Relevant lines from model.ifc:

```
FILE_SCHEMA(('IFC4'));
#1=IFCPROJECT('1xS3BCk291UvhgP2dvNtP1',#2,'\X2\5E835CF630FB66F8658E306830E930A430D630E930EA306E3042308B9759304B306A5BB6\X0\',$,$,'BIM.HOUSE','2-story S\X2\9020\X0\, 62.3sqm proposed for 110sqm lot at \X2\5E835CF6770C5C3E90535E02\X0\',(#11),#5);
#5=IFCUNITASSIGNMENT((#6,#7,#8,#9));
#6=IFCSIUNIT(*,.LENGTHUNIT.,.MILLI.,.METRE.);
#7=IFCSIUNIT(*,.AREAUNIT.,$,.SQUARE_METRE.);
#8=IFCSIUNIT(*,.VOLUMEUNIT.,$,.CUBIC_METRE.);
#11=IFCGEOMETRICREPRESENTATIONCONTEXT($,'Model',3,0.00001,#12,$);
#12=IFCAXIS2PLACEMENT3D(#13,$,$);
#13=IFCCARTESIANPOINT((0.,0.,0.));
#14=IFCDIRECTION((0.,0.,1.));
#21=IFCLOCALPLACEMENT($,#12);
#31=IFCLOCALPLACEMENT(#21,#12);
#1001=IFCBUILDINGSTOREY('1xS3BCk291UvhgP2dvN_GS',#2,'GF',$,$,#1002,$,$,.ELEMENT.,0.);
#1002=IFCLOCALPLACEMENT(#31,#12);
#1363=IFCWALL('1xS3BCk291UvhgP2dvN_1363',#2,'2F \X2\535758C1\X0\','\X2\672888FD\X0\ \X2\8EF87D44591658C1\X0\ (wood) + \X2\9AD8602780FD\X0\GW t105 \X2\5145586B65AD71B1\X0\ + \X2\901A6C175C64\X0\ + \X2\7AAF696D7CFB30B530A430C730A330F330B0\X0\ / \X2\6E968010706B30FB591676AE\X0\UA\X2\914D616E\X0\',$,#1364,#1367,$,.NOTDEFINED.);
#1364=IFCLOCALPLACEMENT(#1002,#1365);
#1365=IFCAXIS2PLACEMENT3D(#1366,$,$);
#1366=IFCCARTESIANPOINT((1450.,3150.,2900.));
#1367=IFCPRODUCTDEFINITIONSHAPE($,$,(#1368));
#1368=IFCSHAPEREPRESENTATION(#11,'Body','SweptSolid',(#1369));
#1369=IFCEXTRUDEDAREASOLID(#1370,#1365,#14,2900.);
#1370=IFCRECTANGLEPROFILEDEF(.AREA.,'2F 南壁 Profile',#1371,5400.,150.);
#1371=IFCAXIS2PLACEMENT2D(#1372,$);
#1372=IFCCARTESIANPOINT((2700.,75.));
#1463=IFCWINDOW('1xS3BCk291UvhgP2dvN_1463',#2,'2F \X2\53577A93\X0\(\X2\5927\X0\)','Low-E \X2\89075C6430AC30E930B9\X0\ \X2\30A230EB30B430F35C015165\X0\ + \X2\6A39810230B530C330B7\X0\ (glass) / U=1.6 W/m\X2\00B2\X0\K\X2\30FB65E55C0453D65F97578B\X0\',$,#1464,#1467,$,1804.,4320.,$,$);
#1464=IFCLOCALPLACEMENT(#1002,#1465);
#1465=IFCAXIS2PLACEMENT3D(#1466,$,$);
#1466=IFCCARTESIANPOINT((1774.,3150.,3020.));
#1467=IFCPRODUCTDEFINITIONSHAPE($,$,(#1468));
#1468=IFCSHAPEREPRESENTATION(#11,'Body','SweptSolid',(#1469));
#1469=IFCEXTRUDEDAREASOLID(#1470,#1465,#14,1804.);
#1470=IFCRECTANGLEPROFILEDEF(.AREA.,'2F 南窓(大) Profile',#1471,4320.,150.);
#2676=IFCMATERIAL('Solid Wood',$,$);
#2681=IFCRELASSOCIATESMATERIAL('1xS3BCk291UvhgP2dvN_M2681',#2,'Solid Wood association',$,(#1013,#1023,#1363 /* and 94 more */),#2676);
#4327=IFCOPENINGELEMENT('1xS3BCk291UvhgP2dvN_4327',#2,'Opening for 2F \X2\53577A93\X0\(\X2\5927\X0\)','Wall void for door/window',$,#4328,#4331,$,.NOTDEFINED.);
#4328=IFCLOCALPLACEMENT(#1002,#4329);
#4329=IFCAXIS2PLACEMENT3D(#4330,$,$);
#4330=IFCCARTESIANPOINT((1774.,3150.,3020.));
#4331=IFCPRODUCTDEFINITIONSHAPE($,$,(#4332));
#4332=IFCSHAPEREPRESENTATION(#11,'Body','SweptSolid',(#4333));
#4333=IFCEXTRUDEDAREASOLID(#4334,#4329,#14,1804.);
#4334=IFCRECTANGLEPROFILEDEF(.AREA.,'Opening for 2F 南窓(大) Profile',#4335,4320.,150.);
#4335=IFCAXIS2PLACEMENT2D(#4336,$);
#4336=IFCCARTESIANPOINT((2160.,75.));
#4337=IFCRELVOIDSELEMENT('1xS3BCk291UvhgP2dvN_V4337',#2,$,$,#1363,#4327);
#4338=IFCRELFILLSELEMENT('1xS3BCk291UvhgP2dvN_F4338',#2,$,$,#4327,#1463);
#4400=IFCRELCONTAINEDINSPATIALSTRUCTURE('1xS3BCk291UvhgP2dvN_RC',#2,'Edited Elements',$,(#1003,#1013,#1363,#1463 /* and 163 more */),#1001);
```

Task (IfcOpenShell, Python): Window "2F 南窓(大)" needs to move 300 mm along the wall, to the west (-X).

```python
import ifcopenshell
import ifcopenshell.api.geometry
import ifcopenshell.util.placement
import ifcopenshell.util.unit

model = ifcopenshell.open("model.ifc")
unit_scale = ifcopenshell.util.unit.calculate_unit_scale(model)

window = model.by_guid("1xS3BCk291UvhgP2dvN_1463")
opening = window.FillsVoids[0].RelatingOpeningElement
wall = opening.VoidsElements[0].RelatingBuildingElement

wall_matrix = ifcopenshell.util.placement.get_local_placement(wall.ObjectPlacement)
shift = wall_matrix[:3, 0] * -0.3 / unit_scale
before = ifcopenshell.util.placement.get_local_placement(window.ObjectPlacement)[:3, 3].copy()

# The window is not placed relative to its opening, so move both.
for product in (opening, window):
    matrix = ifcopenshell.util.placement.get_local_placement(product.ObjectPlacement)
    matrix[:3, 3] += shift
    ifcopenshell.api.geometry.edit_object_placement(model, product=product, matrix=matrix, is_si=False)

after = ifcopenshell.util.placement.get_local_placement(window.ObjectPlacement)[:3, 3]
print("window moved by", (after - before).round(3) + 0.0)

model.write("model-out.ifc")
```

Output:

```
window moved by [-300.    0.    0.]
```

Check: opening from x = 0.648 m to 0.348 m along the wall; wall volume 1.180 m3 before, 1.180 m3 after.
